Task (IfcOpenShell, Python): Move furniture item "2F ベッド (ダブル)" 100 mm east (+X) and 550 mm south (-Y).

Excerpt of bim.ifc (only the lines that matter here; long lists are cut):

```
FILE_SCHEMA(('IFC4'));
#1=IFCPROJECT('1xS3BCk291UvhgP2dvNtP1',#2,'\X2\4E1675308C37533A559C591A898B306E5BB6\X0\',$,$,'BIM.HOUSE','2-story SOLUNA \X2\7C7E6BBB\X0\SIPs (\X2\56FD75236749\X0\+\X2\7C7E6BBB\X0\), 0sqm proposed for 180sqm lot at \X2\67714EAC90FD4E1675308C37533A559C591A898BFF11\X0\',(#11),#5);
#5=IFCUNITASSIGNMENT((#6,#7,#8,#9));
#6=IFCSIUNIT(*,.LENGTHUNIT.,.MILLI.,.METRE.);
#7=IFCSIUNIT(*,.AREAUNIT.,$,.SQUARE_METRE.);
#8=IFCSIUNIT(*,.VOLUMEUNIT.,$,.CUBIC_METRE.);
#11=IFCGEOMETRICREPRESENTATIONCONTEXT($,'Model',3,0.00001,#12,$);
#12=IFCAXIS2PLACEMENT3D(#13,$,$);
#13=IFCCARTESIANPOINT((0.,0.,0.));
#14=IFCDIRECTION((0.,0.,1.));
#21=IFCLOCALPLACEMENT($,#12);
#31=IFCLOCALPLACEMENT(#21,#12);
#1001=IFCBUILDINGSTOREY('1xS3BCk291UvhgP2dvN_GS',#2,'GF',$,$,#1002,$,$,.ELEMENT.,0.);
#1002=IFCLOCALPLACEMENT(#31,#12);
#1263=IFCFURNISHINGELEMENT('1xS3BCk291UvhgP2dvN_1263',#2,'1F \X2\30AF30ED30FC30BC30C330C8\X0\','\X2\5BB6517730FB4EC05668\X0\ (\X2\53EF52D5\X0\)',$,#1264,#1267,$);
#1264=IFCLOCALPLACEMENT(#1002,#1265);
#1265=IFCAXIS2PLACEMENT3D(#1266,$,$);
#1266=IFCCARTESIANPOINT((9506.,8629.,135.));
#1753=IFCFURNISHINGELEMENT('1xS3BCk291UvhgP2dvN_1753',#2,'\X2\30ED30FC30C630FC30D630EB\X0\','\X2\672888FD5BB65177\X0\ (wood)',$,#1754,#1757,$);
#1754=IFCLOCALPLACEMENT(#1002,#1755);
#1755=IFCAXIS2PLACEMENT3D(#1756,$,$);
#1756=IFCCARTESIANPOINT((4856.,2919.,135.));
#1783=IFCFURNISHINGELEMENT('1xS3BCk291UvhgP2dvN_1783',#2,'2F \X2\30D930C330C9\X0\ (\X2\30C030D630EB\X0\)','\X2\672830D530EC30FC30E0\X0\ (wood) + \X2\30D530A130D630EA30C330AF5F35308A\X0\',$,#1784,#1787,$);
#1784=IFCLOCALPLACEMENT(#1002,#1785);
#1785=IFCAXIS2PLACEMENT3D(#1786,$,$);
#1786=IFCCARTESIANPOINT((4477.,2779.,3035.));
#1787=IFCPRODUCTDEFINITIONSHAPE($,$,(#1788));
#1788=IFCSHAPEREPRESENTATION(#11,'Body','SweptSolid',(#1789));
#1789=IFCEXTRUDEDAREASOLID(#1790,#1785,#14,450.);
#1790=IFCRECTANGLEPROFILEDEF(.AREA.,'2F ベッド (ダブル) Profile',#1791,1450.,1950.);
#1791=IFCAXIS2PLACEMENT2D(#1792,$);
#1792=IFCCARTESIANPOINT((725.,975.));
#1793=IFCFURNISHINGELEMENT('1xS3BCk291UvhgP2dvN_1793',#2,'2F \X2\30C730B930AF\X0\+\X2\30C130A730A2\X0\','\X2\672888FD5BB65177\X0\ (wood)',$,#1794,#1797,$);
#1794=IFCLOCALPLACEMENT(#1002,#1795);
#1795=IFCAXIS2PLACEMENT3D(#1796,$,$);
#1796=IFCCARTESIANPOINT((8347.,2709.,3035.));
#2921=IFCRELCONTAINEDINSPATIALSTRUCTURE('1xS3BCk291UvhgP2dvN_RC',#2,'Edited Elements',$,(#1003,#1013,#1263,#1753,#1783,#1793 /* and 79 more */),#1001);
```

```python
import ifcopenshell
import ifcopenshell.api.geometry
import ifcopenshell.util.placement
import ifcopenshell.util.unit

model = ifcopenshell.open("bim.ifc")
unit_scale = ifcopenshell.util.unit.calculate_unit_scale(model)

item = model.by_id(1783)
matrix = ifcopenshell.util.placement.get_local_placement(item.ObjectPlacement)
matrix[0, 3] += 0.1 / unit_scale
matrix[1, 3] -= 0.55 / unit_scale
ifcopenshell.api.geometry.edit_object_placement(model, product=item, matrix=matrix, is_si=False)

print(ifcopenshell.util.placement.get_local_placement(item.ObjectPlacement).round(3) + 0.0)

model.write("bim-out.ifc")
```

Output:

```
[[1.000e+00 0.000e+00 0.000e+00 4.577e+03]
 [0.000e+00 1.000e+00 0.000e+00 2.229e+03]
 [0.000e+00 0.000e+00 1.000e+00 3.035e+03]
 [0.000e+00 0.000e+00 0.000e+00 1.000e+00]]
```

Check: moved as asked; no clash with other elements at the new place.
